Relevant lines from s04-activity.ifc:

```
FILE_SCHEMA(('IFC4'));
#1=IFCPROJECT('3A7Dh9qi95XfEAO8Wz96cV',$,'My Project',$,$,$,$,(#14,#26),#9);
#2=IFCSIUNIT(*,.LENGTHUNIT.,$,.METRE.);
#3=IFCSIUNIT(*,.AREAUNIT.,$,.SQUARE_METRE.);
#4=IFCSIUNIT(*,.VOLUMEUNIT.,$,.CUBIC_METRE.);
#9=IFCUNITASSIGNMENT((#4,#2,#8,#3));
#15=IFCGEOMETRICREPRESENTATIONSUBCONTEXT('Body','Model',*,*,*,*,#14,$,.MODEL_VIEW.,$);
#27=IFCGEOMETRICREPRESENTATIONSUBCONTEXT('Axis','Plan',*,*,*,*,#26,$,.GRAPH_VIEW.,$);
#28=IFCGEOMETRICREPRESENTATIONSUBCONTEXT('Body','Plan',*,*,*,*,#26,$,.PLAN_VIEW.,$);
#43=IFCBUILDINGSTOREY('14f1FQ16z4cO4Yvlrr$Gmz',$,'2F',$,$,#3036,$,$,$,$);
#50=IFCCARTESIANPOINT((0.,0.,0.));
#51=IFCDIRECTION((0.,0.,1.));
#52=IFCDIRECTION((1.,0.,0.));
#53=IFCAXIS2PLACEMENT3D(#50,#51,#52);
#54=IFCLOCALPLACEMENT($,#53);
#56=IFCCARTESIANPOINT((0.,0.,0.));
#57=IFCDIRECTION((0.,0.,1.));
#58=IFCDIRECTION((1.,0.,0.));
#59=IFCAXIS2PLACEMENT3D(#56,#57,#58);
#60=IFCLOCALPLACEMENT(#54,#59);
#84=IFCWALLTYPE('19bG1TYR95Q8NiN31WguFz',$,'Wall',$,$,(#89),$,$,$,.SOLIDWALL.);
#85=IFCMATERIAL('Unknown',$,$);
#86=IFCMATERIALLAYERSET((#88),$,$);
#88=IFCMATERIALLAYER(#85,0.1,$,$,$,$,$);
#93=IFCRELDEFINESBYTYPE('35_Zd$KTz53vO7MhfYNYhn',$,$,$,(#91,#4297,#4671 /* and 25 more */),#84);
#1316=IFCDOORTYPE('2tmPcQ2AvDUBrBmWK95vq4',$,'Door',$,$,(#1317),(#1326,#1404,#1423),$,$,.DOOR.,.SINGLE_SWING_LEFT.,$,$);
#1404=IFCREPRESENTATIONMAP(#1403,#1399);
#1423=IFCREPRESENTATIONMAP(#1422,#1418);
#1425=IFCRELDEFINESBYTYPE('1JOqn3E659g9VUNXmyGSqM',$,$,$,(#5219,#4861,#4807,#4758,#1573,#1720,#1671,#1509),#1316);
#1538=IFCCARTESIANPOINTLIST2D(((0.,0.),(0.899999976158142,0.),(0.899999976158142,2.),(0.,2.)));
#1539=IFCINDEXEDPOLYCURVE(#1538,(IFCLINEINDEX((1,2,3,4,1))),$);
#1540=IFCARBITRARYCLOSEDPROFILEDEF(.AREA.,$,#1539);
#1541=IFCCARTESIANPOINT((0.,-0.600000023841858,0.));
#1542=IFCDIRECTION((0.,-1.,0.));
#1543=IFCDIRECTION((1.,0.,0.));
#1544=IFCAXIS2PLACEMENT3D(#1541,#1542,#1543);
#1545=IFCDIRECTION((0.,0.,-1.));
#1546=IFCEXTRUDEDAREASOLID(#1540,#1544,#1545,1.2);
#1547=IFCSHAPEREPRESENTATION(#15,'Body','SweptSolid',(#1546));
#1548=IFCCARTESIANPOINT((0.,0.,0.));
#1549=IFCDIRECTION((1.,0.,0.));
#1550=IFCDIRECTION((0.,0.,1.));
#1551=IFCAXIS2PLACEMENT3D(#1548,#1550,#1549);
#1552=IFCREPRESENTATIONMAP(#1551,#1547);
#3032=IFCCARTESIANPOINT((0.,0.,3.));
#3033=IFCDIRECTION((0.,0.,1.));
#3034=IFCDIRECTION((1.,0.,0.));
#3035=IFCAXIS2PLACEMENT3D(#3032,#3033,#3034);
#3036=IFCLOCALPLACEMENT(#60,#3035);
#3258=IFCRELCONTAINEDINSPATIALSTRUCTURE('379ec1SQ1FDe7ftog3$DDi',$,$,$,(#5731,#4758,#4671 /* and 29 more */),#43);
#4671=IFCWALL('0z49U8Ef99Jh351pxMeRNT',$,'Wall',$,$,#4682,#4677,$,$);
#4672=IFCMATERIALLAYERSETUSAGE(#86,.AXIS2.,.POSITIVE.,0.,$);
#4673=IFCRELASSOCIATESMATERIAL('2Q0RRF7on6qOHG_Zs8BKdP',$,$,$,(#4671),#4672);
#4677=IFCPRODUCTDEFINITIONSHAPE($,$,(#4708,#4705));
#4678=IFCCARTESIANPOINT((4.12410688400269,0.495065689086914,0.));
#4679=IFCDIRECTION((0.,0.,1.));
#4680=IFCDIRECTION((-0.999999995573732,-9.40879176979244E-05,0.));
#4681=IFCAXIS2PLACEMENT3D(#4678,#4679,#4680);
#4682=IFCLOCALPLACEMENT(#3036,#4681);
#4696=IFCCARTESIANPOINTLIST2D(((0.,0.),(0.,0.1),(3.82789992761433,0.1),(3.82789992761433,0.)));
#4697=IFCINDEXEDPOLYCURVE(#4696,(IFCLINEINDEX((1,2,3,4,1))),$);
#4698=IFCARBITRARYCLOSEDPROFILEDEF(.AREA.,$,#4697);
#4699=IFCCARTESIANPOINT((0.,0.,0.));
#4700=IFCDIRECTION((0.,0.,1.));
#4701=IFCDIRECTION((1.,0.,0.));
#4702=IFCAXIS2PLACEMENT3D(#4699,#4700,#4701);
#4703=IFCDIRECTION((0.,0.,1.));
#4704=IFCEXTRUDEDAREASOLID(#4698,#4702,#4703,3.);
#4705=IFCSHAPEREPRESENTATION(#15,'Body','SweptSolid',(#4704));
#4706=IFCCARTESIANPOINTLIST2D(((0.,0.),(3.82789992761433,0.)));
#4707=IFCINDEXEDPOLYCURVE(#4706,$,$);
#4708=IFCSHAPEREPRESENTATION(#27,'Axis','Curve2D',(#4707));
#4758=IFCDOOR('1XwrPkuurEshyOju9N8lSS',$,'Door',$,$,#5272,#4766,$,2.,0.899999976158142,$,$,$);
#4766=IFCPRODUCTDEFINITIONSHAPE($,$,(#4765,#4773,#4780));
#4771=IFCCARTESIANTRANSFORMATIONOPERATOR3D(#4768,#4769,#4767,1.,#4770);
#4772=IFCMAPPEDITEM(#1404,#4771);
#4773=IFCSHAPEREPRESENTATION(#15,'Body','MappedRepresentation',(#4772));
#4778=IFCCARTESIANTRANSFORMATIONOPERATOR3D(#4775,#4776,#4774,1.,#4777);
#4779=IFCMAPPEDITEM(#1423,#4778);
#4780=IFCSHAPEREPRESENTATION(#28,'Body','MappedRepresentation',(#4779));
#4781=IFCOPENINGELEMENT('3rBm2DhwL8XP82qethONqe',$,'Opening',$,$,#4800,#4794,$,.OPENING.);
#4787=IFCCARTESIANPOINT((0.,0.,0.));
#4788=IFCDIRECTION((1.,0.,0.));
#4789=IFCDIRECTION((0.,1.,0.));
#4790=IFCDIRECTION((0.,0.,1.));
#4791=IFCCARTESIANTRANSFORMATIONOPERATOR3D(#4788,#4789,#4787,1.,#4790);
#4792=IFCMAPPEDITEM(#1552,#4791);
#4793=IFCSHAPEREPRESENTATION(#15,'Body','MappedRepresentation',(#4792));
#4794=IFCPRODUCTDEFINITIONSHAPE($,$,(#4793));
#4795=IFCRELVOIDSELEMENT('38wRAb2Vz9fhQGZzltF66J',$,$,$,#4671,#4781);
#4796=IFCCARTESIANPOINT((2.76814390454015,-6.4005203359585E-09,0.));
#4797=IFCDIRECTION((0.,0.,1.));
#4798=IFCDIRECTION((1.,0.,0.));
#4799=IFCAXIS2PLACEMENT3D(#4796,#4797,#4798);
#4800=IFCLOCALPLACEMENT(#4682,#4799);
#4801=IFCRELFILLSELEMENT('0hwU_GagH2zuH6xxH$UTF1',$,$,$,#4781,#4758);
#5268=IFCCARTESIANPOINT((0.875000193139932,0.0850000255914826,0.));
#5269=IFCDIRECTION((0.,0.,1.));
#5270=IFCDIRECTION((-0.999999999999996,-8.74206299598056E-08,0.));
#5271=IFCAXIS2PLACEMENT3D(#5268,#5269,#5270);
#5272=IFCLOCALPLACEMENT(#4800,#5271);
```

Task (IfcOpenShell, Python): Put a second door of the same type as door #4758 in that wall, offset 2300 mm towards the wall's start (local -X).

```python
import ifcopenshell
import ifcopenshell.api.feature
import ifcopenshell.api.geometry
import ifcopenshell.api.root
import ifcopenshell.geom
import ifcopenshell.util.element
import ifcopenshell.util.placement
import ifcopenshell.util.shape
import ifcopenshell.util.unit

model = ifcopenshell.open("s04-activity.ifc")
unit_scale = ifcopenshell.util.unit.calculate_unit_scale(model)
settings = ifcopenshell.geom.settings()


def volume(element):
    """Net volume in cubic metres, openings subtracted."""
    shape = ifcopenshell.geom.create_shape(settings, element)
    return ifcopenshell.util.shape.get_volume(shape.geometry)


door = model.by_id(4758)
opening = door.FillsVoids[0].RelatingOpeningElement
wall = opening.VoidsElements[0].RelatingBuildingElement
before = volume(wall)
shift = ifcopenshell.util.placement.get_local_placement(wall.ObjectPlacement)[:3, 0] * -2.3 / unit_scale

# copy_class copies the void relationship, type, container and properties, but no geometry.
new_opening = ifcopenshell.api.root.copy_class(model, product=opening)
new_opening.Representation = ifcopenshell.util.element.copy_deep(
    model, opening.Representation, exclude=["IfcGeometricRepresentationContext", "IfcRepresentationMap"]
)
new_door = ifcopenshell.api.root.copy_class(model, product=door)
new_door.Representation = ifcopenshell.util.element.copy_deep(
    model, door.Representation, exclude=["IfcGeometricRepresentationContext", "IfcRepresentationMap"]
)
ifcopenshell.api.feature.add_filling(model, opening=new_opening, element=new_door)

for old, new in ((opening, new_opening), (door, new_door)):
    matrix = ifcopenshell.util.placement.get_local_placement(old.ObjectPlacement)
    matrix[:3, 3] += shift
    ifcopenshell.api.geometry.edit_object_placement(model, product=new, matrix=matrix, is_si=False)

after = volume(wall)

print(f"wall volume {before:.3f} -> {after:.3f} m3")

model.write("s04-activity_edited.ifc")
```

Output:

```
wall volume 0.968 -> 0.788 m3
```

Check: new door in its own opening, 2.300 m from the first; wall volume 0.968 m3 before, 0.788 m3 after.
